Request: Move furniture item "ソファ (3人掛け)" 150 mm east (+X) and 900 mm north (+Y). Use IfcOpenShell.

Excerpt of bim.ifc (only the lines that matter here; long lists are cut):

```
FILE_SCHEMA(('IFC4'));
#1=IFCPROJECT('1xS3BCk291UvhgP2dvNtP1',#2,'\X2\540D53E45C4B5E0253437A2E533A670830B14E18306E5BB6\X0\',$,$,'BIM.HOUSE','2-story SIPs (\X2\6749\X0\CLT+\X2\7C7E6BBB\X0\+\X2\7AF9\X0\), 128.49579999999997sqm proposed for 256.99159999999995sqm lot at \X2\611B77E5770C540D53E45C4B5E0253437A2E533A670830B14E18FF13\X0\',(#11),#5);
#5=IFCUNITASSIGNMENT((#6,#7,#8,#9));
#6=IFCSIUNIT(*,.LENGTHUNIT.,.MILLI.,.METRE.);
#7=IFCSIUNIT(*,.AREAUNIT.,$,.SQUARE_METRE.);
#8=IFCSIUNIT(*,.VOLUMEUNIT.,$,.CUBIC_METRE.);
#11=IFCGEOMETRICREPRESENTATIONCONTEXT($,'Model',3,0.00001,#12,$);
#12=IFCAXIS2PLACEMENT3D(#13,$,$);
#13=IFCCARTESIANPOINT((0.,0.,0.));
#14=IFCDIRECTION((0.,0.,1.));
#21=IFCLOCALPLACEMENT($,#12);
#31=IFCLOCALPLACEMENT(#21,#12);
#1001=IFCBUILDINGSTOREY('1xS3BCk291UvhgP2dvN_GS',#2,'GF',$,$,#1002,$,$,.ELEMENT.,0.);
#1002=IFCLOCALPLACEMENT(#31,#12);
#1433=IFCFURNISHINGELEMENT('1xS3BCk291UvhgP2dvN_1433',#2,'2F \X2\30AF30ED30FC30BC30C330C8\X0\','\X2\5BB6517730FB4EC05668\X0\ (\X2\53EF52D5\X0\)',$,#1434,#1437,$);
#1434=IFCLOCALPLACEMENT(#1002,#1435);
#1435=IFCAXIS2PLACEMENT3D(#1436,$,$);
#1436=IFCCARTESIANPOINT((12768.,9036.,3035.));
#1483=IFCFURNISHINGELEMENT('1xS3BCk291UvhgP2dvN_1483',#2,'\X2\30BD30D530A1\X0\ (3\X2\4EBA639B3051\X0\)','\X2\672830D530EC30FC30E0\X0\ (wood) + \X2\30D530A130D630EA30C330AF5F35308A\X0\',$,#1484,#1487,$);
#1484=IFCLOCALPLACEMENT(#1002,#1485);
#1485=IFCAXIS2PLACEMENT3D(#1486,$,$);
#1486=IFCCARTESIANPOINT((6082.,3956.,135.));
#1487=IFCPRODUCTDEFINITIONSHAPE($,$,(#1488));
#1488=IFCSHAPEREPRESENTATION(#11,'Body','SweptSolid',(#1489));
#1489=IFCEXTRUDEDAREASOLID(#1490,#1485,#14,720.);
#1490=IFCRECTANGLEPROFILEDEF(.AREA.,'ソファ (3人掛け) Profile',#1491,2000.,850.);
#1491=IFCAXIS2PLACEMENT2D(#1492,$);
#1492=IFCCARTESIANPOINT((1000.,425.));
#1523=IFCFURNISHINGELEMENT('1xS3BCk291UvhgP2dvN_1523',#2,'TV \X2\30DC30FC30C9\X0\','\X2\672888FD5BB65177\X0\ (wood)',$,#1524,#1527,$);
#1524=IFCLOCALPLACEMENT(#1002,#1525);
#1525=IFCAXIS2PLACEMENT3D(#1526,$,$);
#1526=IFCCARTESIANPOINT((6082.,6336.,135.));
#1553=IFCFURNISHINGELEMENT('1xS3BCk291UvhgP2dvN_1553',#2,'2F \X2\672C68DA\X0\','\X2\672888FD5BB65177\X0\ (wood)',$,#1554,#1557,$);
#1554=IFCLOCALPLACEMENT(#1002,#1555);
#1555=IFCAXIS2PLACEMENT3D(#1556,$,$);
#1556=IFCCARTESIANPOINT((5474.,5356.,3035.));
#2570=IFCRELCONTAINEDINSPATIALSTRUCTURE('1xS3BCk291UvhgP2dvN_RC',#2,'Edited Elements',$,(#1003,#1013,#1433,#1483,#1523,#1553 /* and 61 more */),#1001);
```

```python
import ifcopenshell
import ifcopenshell.api.geometry
import ifcopenshell.util.placement
import ifcopenshell.util.unit

model = ifcopenshell.open("bim.ifc")
unit_scale = ifcopenshell.util.unit.calculate_unit_scale(model)

item = model.by_id(1483)
matrix = ifcopenshell.util.placement.get_local_placement(item.ObjectPlacement)
matrix[0, 3] += 0.15 / unit_scale
matrix[1, 3] += 0.9 / unit_scale
ifcopenshell.api.geometry.edit_object_placement(model, product=item, matrix=matrix, is_si=False)

print(ifcopenshell.util.placement.get_local_placement(item.ObjectPlacement).round(3) + 0.0)

model.write("bim-out.ifc")
```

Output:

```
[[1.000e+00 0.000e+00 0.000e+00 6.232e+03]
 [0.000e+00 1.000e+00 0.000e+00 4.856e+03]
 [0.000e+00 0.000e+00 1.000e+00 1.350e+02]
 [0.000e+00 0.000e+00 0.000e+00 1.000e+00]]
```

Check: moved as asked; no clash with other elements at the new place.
